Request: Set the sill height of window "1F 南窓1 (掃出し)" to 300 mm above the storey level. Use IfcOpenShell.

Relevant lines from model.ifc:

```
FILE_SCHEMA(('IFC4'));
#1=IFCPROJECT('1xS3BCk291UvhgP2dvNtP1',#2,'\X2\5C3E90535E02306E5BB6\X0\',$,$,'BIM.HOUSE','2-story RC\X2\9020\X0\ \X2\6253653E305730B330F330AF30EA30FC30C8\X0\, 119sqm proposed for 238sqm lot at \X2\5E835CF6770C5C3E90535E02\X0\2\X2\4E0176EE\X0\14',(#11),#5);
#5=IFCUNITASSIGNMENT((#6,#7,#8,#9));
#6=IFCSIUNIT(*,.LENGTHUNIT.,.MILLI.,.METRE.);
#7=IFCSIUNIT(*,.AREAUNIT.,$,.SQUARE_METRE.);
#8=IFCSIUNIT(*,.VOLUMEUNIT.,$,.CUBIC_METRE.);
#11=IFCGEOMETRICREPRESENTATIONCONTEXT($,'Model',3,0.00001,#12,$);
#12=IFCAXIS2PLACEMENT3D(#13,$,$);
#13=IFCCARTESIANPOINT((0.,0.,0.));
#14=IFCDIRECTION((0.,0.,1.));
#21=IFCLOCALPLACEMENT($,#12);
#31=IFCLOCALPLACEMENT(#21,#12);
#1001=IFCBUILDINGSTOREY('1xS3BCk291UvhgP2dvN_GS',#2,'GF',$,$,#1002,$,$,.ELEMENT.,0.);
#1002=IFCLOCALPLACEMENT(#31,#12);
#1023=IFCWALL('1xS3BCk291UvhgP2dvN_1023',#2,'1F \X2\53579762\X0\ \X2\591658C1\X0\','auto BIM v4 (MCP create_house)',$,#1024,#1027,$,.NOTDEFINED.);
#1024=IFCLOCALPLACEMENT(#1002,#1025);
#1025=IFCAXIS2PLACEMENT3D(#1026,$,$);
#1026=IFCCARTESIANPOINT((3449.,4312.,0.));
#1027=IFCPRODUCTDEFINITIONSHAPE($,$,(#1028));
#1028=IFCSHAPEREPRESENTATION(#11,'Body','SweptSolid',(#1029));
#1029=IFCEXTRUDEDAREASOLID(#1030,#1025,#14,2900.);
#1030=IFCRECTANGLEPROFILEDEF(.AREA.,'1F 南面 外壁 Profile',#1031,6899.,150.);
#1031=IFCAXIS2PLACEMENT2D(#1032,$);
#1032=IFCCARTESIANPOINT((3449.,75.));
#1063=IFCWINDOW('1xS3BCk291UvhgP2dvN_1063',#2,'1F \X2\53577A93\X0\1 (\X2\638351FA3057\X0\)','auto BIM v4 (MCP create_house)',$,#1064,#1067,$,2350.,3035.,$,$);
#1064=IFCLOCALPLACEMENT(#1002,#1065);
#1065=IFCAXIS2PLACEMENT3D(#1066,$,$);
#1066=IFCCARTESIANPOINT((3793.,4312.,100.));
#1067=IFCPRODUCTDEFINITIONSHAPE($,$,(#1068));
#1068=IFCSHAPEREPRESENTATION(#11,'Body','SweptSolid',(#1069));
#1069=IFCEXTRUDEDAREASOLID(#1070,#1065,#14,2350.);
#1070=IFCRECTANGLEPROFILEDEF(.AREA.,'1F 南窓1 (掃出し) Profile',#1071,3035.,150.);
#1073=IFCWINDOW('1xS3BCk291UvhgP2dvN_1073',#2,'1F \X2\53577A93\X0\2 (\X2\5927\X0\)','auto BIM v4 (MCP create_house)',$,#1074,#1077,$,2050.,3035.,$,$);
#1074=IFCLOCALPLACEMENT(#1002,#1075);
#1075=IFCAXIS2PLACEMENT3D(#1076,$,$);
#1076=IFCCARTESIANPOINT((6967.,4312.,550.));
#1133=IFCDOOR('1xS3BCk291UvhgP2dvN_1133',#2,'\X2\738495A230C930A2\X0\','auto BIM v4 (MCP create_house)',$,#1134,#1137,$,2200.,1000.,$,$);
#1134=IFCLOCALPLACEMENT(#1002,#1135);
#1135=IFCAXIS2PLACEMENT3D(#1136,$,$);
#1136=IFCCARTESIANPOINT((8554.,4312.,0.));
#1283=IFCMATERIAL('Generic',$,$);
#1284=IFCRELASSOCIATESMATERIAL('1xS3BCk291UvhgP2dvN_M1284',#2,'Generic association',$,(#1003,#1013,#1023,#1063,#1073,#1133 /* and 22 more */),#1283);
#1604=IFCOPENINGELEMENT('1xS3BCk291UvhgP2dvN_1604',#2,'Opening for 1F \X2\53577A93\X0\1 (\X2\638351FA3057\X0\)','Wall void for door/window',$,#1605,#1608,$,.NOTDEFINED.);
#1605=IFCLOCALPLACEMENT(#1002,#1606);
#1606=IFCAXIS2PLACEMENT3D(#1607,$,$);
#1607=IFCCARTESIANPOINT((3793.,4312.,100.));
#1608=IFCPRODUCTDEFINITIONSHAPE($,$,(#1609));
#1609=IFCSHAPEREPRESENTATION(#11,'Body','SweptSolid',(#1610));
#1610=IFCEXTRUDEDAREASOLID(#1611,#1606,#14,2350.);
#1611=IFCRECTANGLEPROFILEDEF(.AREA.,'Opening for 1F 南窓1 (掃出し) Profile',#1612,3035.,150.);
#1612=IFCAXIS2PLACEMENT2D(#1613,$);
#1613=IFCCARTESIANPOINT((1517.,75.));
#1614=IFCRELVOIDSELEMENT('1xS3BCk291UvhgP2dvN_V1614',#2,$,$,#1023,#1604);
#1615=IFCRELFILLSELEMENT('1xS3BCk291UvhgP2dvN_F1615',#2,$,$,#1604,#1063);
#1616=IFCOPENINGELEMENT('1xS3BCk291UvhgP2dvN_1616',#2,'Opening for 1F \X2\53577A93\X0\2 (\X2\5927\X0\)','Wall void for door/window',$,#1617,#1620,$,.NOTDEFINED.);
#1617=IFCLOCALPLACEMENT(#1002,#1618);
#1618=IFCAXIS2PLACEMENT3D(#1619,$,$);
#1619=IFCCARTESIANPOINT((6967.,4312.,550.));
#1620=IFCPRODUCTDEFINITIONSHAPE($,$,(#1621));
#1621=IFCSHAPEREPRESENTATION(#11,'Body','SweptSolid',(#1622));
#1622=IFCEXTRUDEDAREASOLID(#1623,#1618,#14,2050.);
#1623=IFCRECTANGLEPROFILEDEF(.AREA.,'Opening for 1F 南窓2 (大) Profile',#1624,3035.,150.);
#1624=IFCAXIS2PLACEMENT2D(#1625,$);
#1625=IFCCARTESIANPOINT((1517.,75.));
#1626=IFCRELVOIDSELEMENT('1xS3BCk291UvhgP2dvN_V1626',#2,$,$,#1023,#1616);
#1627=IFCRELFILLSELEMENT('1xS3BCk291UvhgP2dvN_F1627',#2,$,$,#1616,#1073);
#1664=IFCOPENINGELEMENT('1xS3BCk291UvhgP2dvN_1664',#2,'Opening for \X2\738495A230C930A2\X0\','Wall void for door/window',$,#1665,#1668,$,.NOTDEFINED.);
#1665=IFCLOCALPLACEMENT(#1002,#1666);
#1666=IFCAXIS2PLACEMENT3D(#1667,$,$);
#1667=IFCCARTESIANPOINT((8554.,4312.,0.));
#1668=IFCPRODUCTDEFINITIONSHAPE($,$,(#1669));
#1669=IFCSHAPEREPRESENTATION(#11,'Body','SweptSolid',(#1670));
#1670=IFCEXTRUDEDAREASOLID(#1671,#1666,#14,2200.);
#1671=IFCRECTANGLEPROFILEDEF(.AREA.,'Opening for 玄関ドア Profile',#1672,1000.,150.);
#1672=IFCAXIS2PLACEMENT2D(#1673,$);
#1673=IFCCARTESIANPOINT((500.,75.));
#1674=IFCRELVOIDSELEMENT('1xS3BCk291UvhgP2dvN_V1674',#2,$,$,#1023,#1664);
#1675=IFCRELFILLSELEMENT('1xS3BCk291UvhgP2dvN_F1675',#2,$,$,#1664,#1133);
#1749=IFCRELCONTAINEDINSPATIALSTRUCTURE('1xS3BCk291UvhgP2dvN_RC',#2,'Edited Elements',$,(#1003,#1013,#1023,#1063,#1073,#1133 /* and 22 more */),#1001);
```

```python
import numpy as np
import ifcopenshell
import ifcopenshell.api.geometry
import ifcopenshell.geom
import ifcopenshell.util.element
import ifcopenshell.util.placement
import ifcopenshell.util.shape
import ifcopenshell.util.unit

model = ifcopenshell.open("model.ifc")
unit_scale = ifcopenshell.util.unit.calculate_unit_scale(model)

window = model.by_id(1063)
opening = window.FillsVoids[0].RelatingOpeningElement
storey = ifcopenshell.util.element.get_container(window, ifc_class="IfcBuildingStorey")
level = ifcopenshell.util.placement.get_local_placement(storey.ObjectPlacement)[2, 3]

# The opening's origin need not be at the sill, so measure its lowest point.
shape = ifcopenshell.geom.create_shape(ifcopenshell.geom.settings(), opening)
bottom = ifcopenshell.util.shape.get_shape_bottom_elevation(shape, shape.geometry) / unit_scale
dz = level + 300.0 - bottom

shift = np.array([0.0, 0.0, dz])
# The window is not placed relative to its opening, so move both.
for product in (opening, window):
    matrix = ifcopenshell.util.placement.get_local_placement(product.ObjectPlacement)
    matrix[:3, 3] += shift
    ifcopenshell.api.geometry.edit_object_placement(model, product=product, matrix=matrix, is_si=False)

print(f"moved by {dz * unit_scale:+.3f} m")

model.write("model_v2.ifc")
```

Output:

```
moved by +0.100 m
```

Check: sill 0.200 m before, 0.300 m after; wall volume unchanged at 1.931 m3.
